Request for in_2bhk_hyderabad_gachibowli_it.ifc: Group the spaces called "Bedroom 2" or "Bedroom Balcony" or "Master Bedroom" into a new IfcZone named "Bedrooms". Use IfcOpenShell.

First a look at what the model holds.

```python
import ifcopenshell

model = ifcopenshell.open("in_2bhk_hyderabad_gachibowli_it.ifc")
print(model.schema)
seen = {}
for space in model.by_type("IfcSpace"):
    seen[space.LongName] = seen.get(space.LongName, 0) + 1
for name, count in sorted(seen.items(), key=str):
    print(count, "x", name)
print("zones:", [z.Name for z in model.by_type("IfcZone")][:20])
```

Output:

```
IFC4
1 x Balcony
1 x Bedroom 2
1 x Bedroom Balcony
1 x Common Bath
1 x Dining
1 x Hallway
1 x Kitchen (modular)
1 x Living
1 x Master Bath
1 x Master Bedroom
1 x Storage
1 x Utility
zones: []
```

```python
import ifcopenshell
import ifcopenshell.api.group
import ifcopenshell.api.root

model = ifcopenshell.open("in_2bhk_hyderabad_gachibowli_it.ifc")

names = {"Bedroom 2", "Bedroom Balcony", "Master Bedroom"}
spaces = [s for s in model.by_type("IfcSpace") if s.LongName in names]

zone = ifcopenshell.api.root.create_entity(model, ifc_class="IfcZone", name="Bedrooms")
ifcopenshell.api.group.assign_group(model, products=spaces, group=zone)
print(len(spaces), "spaces in", zone.Name)

model.write("in_2bhk_hyderabad_gachibowli_it_edited.ifc")
```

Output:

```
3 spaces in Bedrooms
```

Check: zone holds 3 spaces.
